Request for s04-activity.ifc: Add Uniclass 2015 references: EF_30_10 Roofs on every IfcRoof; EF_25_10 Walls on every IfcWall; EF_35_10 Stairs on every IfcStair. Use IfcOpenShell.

First a look at what the model holds.

```python
import ifcopenshell

model = ifcopenshell.open("s04-activity.ifc")
print(model.schema)
print("classifications:", [c.Name for c in model.by_type("IfcClassification")])
for ifc_class in ("IfcDoor", "IfcRoof", "IfcStair", "IfcWall", "IfcWindow"):
    print(ifc_class, len(model.by_type(ifc_class)))
```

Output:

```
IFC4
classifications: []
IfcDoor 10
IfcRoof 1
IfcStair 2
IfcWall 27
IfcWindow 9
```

```python
import ifcopenshell
import ifcopenshell.api.classification

model = ifcopenshell.open("s04-activity.ifc")

system = ifcopenshell.api.classification.add_classification(model, classification="Uniclass 2015")

codes = {
    "IfcRoof": ("EF_30_10", "Roofs"),
    "IfcWall": ("EF_25_10", "Walls"),
    "IfcStair": ("EF_35_10", "Stairs"),
}
for ifc_class, (code, name) in codes.items():
    products = model.by_type(ifc_class)
    ifcopenshell.api.classification.add_reference(
        model, products=products, classification=system, identification=code, name=name
    )
    print(code, len(products))

model.write("s04-activity_v2.ifc")
```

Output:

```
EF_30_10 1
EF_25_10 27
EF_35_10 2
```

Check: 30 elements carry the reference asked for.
